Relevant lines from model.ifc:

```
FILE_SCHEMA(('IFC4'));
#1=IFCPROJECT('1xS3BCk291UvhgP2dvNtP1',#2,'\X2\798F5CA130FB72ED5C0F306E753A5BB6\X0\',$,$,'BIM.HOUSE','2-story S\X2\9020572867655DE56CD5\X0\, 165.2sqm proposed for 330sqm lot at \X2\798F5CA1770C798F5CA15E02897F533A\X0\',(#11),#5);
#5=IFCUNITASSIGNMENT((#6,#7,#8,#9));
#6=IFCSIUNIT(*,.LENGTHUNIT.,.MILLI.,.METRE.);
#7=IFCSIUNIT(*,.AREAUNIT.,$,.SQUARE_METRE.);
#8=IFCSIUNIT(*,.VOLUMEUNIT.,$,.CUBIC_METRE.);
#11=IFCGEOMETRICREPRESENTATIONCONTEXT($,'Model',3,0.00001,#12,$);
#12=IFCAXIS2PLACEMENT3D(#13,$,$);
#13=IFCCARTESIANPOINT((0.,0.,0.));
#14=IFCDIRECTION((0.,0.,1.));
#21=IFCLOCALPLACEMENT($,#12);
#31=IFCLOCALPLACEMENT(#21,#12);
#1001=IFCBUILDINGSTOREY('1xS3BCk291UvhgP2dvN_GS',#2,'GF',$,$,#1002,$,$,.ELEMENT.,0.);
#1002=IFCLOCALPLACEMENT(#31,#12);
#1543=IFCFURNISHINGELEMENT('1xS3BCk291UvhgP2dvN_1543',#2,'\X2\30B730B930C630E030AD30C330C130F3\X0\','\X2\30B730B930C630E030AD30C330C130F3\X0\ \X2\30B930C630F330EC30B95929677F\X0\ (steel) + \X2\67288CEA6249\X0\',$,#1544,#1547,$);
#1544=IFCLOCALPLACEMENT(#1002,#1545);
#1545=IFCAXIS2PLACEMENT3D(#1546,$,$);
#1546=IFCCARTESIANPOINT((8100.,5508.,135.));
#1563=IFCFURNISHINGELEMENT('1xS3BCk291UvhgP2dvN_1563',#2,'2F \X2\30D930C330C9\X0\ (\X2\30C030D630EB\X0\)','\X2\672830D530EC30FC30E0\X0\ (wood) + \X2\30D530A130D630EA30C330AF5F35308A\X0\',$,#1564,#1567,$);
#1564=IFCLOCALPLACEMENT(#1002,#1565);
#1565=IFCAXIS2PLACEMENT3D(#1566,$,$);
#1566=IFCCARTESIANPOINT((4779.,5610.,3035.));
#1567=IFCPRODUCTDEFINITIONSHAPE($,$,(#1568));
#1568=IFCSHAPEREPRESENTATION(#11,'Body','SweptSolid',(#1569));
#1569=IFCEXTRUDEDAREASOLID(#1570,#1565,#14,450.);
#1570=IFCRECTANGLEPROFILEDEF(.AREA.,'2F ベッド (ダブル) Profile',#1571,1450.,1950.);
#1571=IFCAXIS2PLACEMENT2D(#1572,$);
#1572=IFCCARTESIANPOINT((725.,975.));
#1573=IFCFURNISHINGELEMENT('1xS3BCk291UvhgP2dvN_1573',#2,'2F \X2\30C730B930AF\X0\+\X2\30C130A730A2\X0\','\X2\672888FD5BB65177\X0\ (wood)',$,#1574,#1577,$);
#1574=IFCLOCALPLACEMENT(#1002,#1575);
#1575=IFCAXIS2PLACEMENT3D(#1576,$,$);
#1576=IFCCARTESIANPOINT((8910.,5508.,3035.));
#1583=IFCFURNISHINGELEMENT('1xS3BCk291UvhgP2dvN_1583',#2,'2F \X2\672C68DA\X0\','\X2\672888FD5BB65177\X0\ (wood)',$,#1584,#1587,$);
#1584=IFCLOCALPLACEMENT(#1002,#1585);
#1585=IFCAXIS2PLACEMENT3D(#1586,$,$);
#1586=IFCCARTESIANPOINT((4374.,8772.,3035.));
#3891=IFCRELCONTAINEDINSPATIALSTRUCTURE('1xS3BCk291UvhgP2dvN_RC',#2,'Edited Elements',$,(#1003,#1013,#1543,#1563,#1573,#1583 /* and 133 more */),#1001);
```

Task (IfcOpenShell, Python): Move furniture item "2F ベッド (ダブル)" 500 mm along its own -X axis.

```python
import ifcopenshell
import ifcopenshell.api.geometry
import ifcopenshell.util.placement
import ifcopenshell.util.unit

model = ifcopenshell.open("model.ifc")
unit_scale = ifcopenshell.util.unit.calculate_unit_scale(model)

item = model.by_guid("1xS3BCk291UvhgP2dvN_1563")
matrix = ifcopenshell.util.placement.get_local_placement(item.ObjectPlacement)
matrix[:3, 3] -= matrix[:3, 0] * 0.5 / unit_scale
ifcopenshell.api.geometry.edit_object_placement(model, product=item, matrix=matrix, is_si=False)

print(ifcopenshell.util.placement.get_local_placement(item.ObjectPlacement).round(3) + 0.0)

model.write("model_updated.ifc")
```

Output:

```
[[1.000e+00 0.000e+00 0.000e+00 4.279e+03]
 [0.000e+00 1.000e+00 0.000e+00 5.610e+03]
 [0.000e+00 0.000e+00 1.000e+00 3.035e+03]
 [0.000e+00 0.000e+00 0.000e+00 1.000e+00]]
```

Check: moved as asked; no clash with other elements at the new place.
